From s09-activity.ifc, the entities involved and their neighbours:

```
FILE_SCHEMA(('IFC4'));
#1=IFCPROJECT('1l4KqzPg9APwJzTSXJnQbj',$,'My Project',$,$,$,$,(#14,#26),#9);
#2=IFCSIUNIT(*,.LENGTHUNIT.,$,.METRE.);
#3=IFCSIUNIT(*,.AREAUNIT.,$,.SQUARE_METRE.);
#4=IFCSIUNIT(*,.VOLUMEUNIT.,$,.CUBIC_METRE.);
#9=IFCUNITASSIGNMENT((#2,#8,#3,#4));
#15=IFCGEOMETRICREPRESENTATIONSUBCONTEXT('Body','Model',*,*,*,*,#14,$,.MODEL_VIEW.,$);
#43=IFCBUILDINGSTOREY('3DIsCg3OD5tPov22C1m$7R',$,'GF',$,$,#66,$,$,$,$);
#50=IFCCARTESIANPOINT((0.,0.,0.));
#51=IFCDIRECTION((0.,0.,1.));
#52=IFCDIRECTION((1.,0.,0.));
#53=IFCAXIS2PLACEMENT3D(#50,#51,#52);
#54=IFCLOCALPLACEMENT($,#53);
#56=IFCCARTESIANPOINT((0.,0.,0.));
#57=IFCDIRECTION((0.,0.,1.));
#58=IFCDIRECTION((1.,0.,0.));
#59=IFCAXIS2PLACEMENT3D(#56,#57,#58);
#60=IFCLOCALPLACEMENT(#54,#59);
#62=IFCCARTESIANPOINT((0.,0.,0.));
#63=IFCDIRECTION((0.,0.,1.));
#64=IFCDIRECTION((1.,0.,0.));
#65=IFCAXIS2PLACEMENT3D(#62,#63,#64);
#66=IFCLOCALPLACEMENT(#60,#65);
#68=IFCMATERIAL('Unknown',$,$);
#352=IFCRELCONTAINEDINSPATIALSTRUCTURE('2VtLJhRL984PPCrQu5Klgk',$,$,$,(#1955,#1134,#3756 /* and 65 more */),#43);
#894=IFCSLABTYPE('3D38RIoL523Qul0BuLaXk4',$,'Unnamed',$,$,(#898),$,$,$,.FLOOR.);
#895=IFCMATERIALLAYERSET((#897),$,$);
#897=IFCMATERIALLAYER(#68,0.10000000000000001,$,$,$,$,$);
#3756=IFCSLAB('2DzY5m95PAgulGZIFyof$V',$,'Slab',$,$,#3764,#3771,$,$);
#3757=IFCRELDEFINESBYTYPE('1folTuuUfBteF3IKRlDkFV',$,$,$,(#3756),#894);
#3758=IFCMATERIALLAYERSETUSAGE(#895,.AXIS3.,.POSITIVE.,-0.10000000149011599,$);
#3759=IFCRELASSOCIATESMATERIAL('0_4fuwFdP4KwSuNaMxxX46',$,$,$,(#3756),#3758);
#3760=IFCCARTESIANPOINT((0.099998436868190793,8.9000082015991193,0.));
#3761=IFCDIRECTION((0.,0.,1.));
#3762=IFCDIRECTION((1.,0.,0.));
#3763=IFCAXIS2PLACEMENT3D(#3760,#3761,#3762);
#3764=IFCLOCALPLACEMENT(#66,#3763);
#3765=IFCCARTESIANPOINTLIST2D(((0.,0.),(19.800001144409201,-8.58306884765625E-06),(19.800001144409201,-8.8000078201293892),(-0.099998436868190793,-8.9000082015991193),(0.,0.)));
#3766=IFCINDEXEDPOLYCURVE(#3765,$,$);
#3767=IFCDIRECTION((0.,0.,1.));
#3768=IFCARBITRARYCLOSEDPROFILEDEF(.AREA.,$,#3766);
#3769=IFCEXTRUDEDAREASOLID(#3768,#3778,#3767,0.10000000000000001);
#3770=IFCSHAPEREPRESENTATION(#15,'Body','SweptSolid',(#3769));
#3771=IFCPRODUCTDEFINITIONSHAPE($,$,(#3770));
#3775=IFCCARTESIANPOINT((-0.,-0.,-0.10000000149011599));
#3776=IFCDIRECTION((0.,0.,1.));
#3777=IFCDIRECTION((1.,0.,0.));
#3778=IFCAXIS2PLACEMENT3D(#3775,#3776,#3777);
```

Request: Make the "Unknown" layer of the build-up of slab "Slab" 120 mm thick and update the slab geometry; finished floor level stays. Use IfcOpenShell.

```python
import ifcopenshell
import ifcopenshell.util.element
import ifcopenshell.util.representation

model = ifcopenshell.open("s09-activity.ifc")

layer_set = model.by_id(895)
layer = next(l for l in layer_set.MaterialLayers if l.Material and l.Material.Name == "Unknown")
change = 0.12 - layer.LayerThickness
layer.LayerThickness += change

# Geometry does not follow the layer set by itself.
slabs = [e for e in ifcopenshell.util.element.get_elements_by_material(model, layer_set) if e.is_a("IfcSlab")]
for slab in sorted(slabs, key=lambda e: e.id()):
    body = ifcopenshell.util.representation.get_representation(slab, "Model", "Body")
    solid = body.Items[0]
    old_depth = solid.Depth
    solid.Depth += change
    # Extruded upwards: lower the start of the extrusion so the top stays.
    x, y, z = solid.Position.Location.Coordinates
    solid.Position.Location = model.createIfcCartesianPoint((x, y, z - change))
    print(slab.id(), f"{old_depth:g} -> {solid.Depth:g}")

# The layers are counted up from the underside, which has moved.
for usage in {ifcopenshell.util.element.get_material(slab) for slab in slabs}:
    usage.OffsetFromReferenceLine -= change

model.write("s09-activity_edited.ifc")
```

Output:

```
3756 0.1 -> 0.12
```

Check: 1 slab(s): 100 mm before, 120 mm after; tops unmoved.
